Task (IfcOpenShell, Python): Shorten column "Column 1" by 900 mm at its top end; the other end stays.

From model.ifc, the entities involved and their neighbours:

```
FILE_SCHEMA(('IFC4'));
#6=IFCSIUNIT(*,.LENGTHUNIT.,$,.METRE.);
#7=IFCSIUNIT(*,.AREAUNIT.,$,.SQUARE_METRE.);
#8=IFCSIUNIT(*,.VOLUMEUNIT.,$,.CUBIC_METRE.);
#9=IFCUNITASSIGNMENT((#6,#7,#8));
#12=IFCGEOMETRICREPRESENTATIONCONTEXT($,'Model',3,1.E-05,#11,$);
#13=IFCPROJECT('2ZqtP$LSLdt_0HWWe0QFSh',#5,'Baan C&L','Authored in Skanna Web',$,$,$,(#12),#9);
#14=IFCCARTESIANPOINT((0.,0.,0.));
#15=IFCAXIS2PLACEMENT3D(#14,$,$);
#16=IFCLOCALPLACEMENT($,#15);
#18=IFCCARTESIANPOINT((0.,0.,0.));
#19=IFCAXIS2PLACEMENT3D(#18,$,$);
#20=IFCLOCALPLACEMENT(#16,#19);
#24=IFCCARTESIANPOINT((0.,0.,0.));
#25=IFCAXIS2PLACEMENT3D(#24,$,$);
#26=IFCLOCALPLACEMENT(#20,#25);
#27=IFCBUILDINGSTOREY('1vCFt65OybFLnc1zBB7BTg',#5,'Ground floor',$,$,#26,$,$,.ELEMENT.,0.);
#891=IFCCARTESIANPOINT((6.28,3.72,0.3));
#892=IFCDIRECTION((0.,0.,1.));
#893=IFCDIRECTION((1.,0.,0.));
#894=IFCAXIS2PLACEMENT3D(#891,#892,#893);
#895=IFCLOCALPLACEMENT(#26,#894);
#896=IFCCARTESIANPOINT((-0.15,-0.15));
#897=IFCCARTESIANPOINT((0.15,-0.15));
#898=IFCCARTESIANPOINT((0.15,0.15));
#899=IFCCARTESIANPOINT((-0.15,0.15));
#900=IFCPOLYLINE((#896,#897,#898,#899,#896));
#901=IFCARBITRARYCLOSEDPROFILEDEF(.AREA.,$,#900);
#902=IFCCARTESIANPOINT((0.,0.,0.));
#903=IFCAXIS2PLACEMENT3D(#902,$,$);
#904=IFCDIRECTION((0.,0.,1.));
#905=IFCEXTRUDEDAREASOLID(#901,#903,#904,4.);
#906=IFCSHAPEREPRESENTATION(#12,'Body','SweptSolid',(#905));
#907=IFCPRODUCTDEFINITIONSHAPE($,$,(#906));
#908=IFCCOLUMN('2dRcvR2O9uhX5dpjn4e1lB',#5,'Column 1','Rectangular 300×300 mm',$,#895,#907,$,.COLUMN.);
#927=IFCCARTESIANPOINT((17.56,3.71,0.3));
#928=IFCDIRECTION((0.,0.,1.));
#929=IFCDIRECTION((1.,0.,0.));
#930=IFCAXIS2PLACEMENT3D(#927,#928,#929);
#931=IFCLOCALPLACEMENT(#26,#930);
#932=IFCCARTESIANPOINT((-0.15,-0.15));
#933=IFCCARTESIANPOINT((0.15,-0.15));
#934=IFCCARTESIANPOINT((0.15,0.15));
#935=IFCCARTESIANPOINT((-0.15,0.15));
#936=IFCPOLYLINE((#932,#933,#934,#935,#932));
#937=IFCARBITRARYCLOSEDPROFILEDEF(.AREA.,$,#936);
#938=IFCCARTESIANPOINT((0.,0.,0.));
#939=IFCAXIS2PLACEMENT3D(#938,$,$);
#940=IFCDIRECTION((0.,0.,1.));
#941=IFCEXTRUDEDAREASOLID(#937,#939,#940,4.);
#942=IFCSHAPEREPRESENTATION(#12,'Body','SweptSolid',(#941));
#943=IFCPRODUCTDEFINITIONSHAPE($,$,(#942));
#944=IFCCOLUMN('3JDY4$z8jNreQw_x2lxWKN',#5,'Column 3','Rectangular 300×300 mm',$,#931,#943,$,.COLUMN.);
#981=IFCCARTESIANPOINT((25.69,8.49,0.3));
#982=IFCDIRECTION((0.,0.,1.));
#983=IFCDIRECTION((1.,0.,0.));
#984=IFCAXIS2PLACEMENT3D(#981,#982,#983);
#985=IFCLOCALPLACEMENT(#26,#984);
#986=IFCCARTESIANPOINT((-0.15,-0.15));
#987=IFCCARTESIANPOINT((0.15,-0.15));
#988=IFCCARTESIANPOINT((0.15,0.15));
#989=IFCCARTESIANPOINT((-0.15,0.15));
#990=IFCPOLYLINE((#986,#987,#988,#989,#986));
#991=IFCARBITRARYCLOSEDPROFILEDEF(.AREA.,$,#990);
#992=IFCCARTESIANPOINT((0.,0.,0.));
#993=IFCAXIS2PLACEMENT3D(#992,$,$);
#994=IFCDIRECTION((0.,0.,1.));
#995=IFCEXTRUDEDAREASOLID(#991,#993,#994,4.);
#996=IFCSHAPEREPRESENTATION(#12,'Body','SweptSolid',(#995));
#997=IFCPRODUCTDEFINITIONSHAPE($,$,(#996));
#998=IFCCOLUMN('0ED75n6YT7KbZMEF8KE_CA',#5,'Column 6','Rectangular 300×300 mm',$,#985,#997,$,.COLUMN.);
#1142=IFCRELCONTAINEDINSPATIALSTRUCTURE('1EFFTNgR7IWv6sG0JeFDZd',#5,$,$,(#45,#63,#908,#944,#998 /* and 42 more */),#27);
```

```python
import ifcopenshell
import ifcopenshell.util.unit

model = ifcopenshell.open("model.ifc")
unit_scale = ifcopenshell.util.unit.calculate_unit_scale(model)

member = model.by_guid("2dRcvR2O9uhX5dpjn4e1lB")
change = -0.9 / unit_scale

# The extrusion runs towards the end named, so only its depth changes.
body = next(r for r in member.Representation.Representations if r.RepresentationIdentifier == "Body")
solid = body.Items[0]
old_length = solid.Depth
solid.Depth += change

print(f"length {old_length:g} -> {solid.Depth:g}")

model.write("model_edited.ifc")
```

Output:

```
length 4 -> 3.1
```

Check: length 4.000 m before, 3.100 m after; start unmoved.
